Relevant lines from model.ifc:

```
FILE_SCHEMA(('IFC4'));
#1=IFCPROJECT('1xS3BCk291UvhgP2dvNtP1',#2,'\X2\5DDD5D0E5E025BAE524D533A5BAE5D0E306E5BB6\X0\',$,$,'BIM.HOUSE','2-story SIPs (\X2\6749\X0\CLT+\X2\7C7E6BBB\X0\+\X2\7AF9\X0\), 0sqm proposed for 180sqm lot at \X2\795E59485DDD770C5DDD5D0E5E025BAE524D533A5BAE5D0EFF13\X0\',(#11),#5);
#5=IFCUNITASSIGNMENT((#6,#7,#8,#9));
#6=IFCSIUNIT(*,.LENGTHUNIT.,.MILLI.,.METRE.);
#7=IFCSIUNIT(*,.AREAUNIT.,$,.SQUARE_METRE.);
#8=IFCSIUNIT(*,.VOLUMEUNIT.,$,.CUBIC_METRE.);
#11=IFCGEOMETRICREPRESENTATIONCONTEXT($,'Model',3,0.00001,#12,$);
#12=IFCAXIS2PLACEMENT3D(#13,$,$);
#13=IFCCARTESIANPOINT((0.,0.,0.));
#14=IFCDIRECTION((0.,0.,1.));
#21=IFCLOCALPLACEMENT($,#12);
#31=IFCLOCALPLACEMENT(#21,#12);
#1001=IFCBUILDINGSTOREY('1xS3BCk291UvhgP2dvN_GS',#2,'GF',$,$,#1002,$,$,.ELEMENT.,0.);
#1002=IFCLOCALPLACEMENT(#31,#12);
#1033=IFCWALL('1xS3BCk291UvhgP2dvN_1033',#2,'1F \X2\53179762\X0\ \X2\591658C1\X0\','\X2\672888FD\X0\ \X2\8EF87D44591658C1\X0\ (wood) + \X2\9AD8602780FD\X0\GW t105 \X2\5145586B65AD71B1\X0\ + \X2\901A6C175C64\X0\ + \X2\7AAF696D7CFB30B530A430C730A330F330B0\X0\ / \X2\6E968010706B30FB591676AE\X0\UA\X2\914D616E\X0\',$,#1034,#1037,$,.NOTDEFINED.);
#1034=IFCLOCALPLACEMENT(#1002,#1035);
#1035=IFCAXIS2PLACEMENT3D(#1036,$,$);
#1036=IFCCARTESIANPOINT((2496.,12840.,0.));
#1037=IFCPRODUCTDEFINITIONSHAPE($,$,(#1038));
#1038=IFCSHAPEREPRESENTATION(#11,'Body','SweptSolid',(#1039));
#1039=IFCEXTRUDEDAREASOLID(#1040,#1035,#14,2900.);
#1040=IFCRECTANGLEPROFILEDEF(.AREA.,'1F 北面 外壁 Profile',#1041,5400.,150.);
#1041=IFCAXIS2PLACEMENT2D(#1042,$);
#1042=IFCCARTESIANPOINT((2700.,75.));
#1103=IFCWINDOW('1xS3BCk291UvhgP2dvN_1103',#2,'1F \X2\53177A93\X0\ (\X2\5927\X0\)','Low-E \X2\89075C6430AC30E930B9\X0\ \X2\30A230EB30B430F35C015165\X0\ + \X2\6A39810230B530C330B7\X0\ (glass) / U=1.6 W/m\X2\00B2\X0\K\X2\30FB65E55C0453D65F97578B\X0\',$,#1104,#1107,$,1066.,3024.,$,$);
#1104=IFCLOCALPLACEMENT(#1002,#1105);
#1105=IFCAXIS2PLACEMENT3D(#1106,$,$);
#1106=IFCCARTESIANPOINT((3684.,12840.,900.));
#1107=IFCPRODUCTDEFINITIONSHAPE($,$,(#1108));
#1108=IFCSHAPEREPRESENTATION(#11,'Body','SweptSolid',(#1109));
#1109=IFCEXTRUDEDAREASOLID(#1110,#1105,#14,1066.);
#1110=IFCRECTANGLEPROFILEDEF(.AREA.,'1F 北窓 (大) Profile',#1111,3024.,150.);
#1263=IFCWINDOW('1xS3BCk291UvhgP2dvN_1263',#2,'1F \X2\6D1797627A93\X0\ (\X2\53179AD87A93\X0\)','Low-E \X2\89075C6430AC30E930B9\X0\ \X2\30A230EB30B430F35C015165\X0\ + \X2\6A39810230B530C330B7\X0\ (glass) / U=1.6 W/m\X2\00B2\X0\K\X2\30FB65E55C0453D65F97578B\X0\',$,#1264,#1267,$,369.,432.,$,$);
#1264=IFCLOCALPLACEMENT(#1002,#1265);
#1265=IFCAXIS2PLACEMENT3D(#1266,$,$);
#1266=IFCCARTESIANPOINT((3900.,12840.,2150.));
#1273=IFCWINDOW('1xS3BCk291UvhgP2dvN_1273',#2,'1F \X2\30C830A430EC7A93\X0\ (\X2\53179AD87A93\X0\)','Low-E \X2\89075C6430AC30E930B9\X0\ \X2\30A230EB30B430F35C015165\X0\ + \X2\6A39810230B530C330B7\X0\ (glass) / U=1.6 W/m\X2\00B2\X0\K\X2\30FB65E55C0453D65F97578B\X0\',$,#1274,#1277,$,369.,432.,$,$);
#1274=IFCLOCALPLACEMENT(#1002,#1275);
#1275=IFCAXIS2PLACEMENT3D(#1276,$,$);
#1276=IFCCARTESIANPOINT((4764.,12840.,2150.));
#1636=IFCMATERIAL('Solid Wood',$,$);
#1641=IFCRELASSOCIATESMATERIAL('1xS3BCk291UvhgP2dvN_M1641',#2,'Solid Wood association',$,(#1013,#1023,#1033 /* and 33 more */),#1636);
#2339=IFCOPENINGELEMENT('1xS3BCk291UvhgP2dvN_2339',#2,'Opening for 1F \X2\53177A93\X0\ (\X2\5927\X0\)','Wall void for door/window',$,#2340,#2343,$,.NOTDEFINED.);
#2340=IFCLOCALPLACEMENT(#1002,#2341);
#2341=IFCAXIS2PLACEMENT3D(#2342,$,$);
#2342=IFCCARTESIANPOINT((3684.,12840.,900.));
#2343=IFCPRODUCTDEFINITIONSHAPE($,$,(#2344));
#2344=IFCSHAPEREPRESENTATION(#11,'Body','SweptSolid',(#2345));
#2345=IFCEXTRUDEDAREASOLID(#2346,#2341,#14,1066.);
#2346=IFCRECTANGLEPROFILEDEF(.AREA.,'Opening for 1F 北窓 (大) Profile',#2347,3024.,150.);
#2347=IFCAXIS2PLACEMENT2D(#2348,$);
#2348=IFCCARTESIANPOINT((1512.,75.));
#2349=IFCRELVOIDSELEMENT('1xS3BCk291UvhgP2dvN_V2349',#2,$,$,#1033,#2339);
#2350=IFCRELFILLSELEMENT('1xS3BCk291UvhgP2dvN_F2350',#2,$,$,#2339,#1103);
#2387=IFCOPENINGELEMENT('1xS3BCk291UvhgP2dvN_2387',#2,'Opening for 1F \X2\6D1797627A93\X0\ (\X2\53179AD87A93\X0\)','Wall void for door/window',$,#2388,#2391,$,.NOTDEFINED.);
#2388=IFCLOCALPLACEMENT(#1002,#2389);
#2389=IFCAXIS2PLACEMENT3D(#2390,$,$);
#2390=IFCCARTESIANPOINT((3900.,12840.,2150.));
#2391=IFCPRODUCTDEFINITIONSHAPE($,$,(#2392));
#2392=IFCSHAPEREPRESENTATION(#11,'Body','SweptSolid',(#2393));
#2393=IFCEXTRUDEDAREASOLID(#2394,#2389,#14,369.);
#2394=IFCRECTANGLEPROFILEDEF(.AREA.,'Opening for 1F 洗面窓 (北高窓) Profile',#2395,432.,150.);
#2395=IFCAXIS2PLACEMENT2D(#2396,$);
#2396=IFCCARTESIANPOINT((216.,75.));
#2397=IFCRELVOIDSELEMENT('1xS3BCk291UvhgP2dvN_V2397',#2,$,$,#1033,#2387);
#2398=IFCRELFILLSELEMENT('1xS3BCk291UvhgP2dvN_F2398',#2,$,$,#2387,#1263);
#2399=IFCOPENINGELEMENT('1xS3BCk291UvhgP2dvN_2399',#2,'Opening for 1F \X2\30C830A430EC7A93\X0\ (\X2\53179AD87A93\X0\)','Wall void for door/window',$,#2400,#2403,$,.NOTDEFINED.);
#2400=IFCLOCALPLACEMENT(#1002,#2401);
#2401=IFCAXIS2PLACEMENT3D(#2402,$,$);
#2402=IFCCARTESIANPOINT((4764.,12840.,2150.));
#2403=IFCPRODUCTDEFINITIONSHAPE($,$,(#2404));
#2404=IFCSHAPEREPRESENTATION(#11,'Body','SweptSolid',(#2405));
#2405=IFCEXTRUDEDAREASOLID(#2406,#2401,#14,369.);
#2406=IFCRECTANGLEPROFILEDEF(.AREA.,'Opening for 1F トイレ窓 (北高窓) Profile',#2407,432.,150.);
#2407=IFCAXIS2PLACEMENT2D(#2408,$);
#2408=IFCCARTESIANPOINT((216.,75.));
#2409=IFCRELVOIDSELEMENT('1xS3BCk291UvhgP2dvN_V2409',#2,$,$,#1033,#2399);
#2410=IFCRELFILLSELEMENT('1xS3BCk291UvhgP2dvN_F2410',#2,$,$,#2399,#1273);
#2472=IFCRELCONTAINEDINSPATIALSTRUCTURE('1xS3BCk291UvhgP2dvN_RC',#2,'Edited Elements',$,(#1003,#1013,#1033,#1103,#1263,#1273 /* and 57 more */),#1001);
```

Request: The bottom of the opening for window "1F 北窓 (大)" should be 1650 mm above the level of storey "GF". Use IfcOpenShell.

```python
import numpy as np
import ifcopenshell
import ifcopenshell.api.geometry
import ifcopenshell.geom
import ifcopenshell.util.element
import ifcopenshell.util.placement
import ifcopenshell.util.shape
import ifcopenshell.util.unit

model = ifcopenshell.open("model.ifc")
unit_scale = ifcopenshell.util.unit.calculate_unit_scale(model)

window = model.by_guid("1xS3BCk291UvhgP2dvN_1103")
opening = window.FillsVoids[0].RelatingOpeningElement
storey = ifcopenshell.util.element.get_container(window, ifc_class="IfcBuildingStorey")
level = ifcopenshell.util.placement.get_local_placement(storey.ObjectPlacement)[2, 3]

# The opening's origin need not be at the sill, so measure its lowest point.
shape = ifcopenshell.geom.create_shape(ifcopenshell.geom.settings(), opening)
bottom = ifcopenshell.util.shape.get_shape_bottom_elevation(shape, shape.geometry) / unit_scale
dz = level + 1650.0 - bottom

shift = np.array([0.0, 0.0, dz])
# The window is not placed relative to its opening, so move both.
for product in (opening, window):
    matrix = ifcopenshell.util.placement.get_local_placement(product.ObjectPlacement)
    matrix[:3, 3] += shift
    ifcopenshell.api.geometry.edit_object_placement(model, product=product, matrix=matrix, is_si=False)

print(f"moved by {dz * unit_scale:+.3f} m")

model.write("model_v2.ifc")
```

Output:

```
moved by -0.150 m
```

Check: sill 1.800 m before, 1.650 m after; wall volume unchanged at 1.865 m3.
